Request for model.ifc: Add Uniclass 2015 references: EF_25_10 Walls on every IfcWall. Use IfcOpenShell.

First a look at what the model holds.

```python
import ifcopenshell

model = ifcopenshell.open("model.ifc")
print(model.schema)
print("classifications:", [c.Name for c in model.by_type("IfcClassification")])
for ifc_class in ("IfcDoor", "IfcRoof", "IfcStair", "IfcWall", "IfcWindow"):
    print(ifc_class, len(model.by_type(ifc_class)))
```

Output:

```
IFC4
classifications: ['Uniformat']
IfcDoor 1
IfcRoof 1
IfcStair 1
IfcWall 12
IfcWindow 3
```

```python
import ifcopenshell
import ifcopenshell.api.classification

model = ifcopenshell.open("model.ifc")

system = ifcopenshell.api.classification.add_classification(model, classification="Uniclass 2015")

codes = {
    "IfcWall": ("EF_25_10", "Walls"),
}
for ifc_class, (code, name) in codes.items():
    products = model.by_type(ifc_class)
    ifcopenshell.api.classification.add_reference(
        model, products=products, classification=system, identification=code, name=name
    )
    print(code, len(products))

model.write("model-out.ifc")
```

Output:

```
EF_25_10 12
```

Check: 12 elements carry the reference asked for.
